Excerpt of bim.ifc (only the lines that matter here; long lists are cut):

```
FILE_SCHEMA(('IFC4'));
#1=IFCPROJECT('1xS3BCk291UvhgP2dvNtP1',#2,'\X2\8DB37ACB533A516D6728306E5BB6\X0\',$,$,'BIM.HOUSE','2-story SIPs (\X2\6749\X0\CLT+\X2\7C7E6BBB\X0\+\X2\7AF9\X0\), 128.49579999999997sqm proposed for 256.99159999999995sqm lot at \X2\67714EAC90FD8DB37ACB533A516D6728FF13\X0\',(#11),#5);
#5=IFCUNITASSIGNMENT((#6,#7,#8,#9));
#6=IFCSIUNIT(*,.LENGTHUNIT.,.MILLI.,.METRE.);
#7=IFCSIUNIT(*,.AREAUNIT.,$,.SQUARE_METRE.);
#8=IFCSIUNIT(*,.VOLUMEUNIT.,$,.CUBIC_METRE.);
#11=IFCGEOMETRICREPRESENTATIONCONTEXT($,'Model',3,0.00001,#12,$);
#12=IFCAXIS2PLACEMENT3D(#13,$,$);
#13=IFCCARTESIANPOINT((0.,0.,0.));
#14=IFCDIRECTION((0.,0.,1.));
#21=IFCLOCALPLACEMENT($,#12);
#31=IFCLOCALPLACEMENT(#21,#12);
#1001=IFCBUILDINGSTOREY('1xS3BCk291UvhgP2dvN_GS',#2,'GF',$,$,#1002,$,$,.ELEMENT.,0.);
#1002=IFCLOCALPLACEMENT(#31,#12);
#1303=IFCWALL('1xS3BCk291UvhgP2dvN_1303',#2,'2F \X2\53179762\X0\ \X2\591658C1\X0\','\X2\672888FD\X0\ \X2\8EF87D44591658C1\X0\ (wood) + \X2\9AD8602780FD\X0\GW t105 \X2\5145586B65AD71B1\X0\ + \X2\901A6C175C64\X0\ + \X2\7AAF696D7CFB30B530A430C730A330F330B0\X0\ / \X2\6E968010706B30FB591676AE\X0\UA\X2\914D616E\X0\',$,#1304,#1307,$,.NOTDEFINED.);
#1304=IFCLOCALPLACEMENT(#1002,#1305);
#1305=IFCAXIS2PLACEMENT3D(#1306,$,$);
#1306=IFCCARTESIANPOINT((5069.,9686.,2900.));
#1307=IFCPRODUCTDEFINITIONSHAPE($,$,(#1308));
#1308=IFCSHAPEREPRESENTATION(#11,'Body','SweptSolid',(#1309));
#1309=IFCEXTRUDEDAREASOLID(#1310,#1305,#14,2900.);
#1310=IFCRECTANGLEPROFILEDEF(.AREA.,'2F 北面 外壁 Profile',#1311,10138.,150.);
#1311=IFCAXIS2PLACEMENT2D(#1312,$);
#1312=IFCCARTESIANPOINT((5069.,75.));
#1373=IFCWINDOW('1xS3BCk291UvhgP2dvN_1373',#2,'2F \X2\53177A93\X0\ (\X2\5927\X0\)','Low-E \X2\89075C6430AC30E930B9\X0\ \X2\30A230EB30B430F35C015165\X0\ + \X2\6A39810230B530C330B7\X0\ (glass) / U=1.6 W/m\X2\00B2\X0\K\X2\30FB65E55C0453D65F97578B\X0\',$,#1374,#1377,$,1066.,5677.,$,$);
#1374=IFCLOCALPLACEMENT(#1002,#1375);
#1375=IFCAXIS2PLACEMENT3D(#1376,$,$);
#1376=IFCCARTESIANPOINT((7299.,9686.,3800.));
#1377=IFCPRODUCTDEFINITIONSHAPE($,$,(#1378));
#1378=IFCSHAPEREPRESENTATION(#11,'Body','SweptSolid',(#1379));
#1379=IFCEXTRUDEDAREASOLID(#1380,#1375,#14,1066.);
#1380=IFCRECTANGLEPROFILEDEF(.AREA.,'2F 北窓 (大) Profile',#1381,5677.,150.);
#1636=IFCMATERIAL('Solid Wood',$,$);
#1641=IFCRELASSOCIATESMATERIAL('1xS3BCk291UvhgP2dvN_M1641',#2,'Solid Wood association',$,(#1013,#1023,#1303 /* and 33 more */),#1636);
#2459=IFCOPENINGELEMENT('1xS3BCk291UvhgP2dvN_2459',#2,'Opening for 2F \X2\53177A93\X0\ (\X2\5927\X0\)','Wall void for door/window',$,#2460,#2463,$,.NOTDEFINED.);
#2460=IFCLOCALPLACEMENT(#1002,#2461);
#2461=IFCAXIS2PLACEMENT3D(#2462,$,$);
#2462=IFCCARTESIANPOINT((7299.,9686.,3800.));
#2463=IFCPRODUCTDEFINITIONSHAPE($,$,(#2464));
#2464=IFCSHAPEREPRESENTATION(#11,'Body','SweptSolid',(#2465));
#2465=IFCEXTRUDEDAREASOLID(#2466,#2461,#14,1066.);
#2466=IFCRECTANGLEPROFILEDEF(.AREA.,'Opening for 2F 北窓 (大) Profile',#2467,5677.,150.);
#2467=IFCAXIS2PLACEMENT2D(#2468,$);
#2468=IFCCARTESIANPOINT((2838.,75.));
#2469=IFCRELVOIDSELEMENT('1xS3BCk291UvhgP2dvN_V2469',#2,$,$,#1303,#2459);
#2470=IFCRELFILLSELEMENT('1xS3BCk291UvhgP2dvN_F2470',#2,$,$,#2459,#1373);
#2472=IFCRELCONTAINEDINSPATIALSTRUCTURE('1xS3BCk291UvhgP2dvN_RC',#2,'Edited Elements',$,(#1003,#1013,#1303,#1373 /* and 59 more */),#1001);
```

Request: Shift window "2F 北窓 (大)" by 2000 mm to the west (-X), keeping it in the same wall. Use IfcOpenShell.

```python
import ifcopenshell
import ifcopenshell.api.geometry
import ifcopenshell.util.placement

model = ifcopenshell.open("bim.ifc")

window = model.by_id(1373)
opening = window.FillsVoids[0].RelatingOpeningElement
wall = opening.VoidsElements[0].RelatingBuildingElement

wall_matrix = ifcopenshell.util.placement.get_local_placement(wall.ObjectPlacement)
shift = wall_matrix[:3, 0] * -2000.0
before = ifcopenshell.util.placement.get_local_placement(window.ObjectPlacement)[:3, 3].copy()

# The window is not placed relative to its opening, so move both.
for product in (opening, window):
    matrix = ifcopenshell.util.placement.get_local_placement(product.ObjectPlacement)
    matrix[:3, 3] += shift
    ifcopenshell.api.geometry.edit_object_placement(model, product=product, matrix=matrix, is_si=False)

after = ifcopenshell.util.placement.get_local_placement(window.ObjectPlacement)[:3, 3]
print("window moved by", (after - before).round(3) + 0.0)

model.write("bim_updated.ifc")
```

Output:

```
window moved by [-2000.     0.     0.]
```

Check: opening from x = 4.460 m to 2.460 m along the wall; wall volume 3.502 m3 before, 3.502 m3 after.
